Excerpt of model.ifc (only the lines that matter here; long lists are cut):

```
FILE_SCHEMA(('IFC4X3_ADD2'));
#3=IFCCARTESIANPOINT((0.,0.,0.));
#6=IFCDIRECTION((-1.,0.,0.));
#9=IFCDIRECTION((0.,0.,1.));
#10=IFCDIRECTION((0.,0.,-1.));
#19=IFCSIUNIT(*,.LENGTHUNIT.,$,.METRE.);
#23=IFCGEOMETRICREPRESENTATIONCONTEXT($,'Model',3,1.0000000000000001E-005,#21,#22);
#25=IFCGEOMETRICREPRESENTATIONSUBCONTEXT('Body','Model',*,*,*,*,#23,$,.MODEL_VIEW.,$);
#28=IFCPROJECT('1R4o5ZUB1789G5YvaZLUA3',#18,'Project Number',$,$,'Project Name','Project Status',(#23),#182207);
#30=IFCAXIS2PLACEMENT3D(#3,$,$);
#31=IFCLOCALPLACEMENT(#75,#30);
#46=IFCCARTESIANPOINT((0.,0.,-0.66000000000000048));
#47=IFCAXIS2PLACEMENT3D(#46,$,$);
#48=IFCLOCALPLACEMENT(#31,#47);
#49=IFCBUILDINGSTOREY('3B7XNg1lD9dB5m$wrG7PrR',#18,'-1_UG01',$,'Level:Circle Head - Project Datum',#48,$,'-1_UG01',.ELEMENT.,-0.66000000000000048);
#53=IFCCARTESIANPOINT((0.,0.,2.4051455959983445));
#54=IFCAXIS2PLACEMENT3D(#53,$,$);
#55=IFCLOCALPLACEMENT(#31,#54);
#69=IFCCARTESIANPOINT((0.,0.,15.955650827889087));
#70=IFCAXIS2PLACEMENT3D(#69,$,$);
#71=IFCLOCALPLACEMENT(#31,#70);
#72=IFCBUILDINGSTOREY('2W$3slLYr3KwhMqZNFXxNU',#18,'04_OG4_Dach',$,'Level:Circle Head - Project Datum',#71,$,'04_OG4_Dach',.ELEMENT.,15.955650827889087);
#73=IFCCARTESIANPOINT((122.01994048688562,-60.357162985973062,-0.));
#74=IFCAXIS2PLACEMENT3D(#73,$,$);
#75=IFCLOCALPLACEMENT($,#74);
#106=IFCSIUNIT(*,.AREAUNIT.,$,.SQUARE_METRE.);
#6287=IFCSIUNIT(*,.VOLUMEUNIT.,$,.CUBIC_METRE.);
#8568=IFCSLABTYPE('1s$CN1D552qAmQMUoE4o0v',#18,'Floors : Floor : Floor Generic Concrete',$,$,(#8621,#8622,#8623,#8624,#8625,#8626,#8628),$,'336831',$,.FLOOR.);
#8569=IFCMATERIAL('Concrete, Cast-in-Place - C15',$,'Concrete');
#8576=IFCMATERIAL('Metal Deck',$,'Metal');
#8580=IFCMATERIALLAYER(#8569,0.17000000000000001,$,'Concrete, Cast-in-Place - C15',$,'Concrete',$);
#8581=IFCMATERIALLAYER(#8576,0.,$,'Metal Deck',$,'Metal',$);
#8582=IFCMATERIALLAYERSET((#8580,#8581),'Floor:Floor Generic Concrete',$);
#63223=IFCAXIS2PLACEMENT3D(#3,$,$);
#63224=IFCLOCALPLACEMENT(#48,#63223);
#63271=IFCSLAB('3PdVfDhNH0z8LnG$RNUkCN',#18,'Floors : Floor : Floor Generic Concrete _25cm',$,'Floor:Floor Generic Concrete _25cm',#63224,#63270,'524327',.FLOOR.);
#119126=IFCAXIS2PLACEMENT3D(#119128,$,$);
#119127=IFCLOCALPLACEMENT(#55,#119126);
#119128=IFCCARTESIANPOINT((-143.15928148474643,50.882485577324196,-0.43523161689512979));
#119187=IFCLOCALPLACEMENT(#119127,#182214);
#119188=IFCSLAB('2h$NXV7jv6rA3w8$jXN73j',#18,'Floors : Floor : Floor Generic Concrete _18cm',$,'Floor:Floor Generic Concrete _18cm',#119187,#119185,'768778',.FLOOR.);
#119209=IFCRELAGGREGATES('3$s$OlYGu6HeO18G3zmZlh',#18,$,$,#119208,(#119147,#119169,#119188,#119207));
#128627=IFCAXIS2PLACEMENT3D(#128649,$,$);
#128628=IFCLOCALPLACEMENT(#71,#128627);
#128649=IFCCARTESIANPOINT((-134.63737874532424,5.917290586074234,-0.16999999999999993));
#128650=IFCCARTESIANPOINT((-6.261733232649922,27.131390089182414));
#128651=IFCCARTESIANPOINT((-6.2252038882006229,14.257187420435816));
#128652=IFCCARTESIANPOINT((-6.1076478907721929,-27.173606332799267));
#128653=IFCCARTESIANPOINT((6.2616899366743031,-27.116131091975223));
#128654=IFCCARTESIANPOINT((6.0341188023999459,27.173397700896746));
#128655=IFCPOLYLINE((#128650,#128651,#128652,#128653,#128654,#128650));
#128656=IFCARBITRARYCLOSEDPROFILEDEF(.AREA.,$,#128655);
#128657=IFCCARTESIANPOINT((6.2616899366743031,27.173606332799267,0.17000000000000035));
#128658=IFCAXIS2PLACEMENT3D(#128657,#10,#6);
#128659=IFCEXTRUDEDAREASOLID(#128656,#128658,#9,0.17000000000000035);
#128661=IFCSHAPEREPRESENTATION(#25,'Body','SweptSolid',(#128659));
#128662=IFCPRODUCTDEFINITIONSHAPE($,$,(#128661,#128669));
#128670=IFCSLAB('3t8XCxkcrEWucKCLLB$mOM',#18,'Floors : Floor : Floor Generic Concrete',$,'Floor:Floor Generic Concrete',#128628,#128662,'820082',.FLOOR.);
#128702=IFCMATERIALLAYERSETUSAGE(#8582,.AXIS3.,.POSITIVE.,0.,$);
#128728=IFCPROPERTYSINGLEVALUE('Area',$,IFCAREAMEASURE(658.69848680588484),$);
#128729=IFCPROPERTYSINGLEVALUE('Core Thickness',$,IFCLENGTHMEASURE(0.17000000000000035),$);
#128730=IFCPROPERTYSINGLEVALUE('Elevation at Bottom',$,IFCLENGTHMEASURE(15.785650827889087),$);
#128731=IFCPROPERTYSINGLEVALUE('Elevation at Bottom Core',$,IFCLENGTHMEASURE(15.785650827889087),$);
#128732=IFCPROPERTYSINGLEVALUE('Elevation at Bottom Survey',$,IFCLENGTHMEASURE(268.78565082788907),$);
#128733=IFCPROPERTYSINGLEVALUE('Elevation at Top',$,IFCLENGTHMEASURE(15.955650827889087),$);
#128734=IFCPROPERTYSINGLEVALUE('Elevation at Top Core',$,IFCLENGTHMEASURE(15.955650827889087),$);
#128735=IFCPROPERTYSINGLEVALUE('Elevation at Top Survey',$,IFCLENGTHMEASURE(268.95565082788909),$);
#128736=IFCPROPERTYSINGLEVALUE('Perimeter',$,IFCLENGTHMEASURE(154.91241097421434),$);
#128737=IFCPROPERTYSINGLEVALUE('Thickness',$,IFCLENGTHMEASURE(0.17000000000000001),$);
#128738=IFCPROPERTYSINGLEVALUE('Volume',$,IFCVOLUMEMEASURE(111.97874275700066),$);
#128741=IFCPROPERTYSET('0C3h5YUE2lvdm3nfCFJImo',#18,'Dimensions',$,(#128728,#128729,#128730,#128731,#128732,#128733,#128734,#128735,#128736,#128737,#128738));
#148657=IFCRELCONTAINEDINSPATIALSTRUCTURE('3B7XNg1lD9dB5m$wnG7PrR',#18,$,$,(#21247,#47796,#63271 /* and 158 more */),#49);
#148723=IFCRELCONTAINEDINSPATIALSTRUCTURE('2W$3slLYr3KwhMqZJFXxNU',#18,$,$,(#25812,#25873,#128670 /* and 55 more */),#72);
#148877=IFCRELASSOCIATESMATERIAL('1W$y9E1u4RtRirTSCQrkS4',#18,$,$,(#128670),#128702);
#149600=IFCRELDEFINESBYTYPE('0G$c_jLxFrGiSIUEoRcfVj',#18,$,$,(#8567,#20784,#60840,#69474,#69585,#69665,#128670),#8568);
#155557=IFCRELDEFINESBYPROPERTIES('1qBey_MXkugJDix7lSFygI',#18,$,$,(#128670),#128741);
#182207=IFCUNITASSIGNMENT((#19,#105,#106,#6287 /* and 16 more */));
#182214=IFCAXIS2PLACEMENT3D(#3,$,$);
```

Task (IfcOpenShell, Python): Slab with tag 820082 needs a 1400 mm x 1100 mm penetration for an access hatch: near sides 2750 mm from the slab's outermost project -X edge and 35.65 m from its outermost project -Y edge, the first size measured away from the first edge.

```python
import numpy as np
import ifcopenshell
import ifcopenshell.api.feature
import ifcopenshell.api.geometry
import ifcopenshell.api.pset
import ifcopenshell.api.root
import ifcopenshell.geom
import ifcopenshell.util.element
import ifcopenshell.util.placement
import ifcopenshell.util.representation
import ifcopenshell.util.shape
import ifcopenshell.util.unit

model = ifcopenshell.open("model.ifc")
unit_scale = ifcopenshell.util.unit.calculate_unit_scale(model)
area_scale = ifcopenshell.util.unit.calculate_unit_scale(model, "AREAUNIT")
volume_scale = ifcopenshell.util.unit.calculate_unit_scale(model, "VOLUMEUNIT")
settings = ifcopenshell.geom.settings()


def volume(element):
    """Net volume in cubic metres, openings subtracted."""
    shape = ifcopenshell.geom.create_shape(settings, element)
    return ifcopenshell.util.shape.get_volume(shape.geometry)


slab = model.by_guid("3t8XCxkcrEWucKCLLB$mOM")
before = volume(slab)

# Extent in the slab's own axes, in metres. The edges named are its -X and -Y sides.
slab_shape = ifcopenshell.geom.create_shape(settings, slab)
vertices = ifcopenshell.util.shape.get_vertices(slab_shape.geometry)
x_min, y_min, bottom = vertices.min(axis=0)
top = vertices[:, 2].max()

opening = ifcopenshell.api.root.create_entity(model, ifc_class="IfcOpeningElement", name="Access hatch opening", predefined_type="OPENING")
context = ifcopenshell.util.representation.get_context(model, "Model", "Body", "MODEL_VIEW")
width, depth = 1.4, 1.1
outline = [(0.0, 0.0), (width, 0.0), (width, depth), (0.0, depth), (0.0, 0.0)]
# Overshoot both faces by 50 mm so the cut is clean.
shape = ifcopenshell.api.geometry.add_slab_representation(
    model, context=context, depth=top - bottom + 0.1, polyline=outline
)
ifcopenshell.api.geometry.assign_representation(model, product=opening, representation=shape)

matrix = ifcopenshell.util.placement.get_local_placement(slab.ObjectPlacement)
matrix[:, 3] = matrix @ np.append(np.array([x_min + 2.75, y_min + 35.65, bottom - 0.05]) / unit_scale, 1.0)
ifcopenshell.api.geometry.edit_object_placement(model, product=opening, matrix=matrix, is_si=False)
ifcopenshell.api.feature.add_feature(model, feature=opening, element=slab)

after = volume(slab)

# Update the slab's stored quantities.
pset = model.by_id(ifcopenshell.util.element.get_pset(slab, "Dimensions", should_inherit=False)["id"])
ifcopenshell.api.pset.edit_pset(model, pset=pset, properties={
    "Area": model.create_entity("IfcAreaMeasure", after / (top - bottom) / area_scale),
    "Volume": model.create_entity("IfcVolumeMeasure", after / volume_scale),
})

print(f"slab volume {before:.3f} -> {after:.3f} m3")

model.write("model_rev.ifc")
```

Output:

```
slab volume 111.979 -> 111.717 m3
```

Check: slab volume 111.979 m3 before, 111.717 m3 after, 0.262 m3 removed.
